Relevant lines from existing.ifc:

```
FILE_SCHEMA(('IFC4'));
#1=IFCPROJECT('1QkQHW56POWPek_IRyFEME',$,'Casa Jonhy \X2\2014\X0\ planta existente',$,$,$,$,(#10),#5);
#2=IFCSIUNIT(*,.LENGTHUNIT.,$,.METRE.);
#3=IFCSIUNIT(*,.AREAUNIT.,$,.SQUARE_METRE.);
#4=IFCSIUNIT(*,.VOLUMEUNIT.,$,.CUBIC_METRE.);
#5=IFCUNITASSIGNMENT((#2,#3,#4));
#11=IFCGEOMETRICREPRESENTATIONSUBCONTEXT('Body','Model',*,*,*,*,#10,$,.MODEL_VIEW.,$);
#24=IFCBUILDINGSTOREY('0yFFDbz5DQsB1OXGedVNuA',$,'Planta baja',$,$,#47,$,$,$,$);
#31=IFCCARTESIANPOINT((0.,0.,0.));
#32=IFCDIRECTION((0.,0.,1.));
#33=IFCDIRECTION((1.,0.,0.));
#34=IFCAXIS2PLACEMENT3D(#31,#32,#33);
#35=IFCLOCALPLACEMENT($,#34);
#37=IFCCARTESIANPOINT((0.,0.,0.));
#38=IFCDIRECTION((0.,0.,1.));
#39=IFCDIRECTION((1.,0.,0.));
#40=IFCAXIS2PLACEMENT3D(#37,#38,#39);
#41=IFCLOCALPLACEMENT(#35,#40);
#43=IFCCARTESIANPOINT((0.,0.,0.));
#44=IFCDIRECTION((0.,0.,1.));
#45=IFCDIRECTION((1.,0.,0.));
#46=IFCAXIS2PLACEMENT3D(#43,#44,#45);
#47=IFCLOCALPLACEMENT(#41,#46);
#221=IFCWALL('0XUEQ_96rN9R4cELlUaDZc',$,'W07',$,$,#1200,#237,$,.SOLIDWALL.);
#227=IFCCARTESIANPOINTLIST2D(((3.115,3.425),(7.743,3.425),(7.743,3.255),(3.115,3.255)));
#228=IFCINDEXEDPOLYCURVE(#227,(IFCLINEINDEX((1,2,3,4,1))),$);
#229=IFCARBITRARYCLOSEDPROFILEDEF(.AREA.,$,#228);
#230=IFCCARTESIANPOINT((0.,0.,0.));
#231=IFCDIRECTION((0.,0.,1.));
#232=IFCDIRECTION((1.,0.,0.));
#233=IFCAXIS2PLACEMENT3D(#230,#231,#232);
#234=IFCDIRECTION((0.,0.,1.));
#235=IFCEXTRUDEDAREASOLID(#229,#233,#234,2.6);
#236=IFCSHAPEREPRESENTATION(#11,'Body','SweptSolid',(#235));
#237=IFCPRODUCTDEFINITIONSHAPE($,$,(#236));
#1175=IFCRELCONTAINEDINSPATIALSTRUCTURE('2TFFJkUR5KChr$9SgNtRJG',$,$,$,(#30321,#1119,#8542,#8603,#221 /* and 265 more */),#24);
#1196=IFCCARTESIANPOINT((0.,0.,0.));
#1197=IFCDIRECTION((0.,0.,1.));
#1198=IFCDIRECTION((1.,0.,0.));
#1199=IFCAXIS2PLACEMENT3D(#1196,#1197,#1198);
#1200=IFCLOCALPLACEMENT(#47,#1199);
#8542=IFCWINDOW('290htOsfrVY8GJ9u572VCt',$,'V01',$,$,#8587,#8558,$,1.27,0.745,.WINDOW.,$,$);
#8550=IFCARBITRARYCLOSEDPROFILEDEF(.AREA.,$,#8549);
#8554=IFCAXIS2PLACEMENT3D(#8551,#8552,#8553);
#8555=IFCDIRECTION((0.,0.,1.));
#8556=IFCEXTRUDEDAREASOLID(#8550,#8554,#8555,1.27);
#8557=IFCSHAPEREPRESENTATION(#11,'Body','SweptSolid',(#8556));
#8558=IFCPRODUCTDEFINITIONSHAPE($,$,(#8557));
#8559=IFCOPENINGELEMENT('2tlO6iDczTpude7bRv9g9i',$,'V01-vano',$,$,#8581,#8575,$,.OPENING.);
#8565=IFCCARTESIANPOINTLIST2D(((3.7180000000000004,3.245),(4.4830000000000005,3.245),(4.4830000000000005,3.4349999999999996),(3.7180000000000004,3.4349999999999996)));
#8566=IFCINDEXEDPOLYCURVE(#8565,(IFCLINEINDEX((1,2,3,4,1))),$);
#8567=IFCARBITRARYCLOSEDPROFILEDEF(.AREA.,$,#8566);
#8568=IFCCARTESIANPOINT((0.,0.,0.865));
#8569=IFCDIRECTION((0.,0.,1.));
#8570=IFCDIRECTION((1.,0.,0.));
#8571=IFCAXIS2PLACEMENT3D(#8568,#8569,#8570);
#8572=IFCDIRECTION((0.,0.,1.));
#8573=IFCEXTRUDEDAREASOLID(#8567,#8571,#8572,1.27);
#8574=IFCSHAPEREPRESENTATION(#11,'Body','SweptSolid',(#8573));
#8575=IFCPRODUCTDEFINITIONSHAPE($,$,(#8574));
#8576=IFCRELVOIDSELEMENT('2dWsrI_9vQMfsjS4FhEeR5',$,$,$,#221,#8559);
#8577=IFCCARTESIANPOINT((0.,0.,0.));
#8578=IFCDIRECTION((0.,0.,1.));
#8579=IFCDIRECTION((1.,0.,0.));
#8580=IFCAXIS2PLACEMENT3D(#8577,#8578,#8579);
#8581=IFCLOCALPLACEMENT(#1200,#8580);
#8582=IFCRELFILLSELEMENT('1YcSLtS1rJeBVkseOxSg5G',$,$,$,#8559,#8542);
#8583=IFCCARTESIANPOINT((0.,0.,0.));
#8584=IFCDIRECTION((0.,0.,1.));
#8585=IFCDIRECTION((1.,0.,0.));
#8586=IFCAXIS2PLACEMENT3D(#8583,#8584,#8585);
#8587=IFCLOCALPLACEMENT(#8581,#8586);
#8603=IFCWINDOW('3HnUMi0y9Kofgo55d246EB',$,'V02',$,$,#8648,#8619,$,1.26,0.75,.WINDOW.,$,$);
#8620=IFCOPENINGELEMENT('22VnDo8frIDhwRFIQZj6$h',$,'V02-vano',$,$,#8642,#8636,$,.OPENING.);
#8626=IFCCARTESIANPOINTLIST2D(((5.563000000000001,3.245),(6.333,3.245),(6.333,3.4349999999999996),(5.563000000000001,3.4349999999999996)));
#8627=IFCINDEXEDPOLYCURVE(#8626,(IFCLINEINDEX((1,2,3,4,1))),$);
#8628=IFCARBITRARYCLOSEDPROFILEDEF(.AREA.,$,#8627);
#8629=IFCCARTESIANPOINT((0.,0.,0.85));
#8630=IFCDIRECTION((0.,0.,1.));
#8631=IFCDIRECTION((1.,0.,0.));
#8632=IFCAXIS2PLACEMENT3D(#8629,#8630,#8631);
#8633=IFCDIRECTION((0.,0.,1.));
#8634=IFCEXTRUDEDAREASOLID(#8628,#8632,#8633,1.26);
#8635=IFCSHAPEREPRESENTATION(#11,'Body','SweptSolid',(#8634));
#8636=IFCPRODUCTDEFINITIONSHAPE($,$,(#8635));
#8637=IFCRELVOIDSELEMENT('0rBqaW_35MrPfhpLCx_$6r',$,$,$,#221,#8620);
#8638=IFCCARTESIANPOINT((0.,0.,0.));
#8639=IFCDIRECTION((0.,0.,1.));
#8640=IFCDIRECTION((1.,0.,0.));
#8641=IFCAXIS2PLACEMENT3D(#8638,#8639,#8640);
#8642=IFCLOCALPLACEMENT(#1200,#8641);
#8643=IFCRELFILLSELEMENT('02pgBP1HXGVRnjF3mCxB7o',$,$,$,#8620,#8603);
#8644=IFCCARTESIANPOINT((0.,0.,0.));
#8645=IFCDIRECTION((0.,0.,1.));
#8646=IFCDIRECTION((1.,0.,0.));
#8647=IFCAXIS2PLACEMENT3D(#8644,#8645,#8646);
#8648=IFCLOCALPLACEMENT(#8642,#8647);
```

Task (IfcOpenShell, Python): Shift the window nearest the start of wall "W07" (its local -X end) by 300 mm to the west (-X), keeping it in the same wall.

```python
import ifcopenshell
import ifcopenshell.api.geometry
import ifcopenshell.util.placement
import ifcopenshell.util.unit

model = ifcopenshell.open("existing.ifc")
unit_scale = ifcopenshell.util.unit.calculate_unit_scale(model)

window = model.by_guid("290htOsfrVY8GJ9u572VCt")
opening = window.FillsVoids[0].RelatingOpeningElement
wall = opening.VoidsElements[0].RelatingBuildingElement

wall_matrix = ifcopenshell.util.placement.get_local_placement(wall.ObjectPlacement)
shift = wall_matrix[:3, 0] * -0.3 / unit_scale
before = ifcopenshell.util.placement.get_local_placement(window.ObjectPlacement)[:3, 3].copy()

# The window is placed relative to its opening, so it follows when the opening moves.
matrix = ifcopenshell.util.placement.get_local_placement(opening.ObjectPlacement)
matrix[:3, 3] += shift
ifcopenshell.api.geometry.edit_object_placement(
    model, product=opening, matrix=matrix, is_si=False, should_transform_children=True
)

after = ifcopenshell.util.placement.get_local_placement(window.ObjectPlacement)[:3, 3]
print("window moved by", (after - before).round(3) + 0.0)

model.write("existing-out.ifc")
```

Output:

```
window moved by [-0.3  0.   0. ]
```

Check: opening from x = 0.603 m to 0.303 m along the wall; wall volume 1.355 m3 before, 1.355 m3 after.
